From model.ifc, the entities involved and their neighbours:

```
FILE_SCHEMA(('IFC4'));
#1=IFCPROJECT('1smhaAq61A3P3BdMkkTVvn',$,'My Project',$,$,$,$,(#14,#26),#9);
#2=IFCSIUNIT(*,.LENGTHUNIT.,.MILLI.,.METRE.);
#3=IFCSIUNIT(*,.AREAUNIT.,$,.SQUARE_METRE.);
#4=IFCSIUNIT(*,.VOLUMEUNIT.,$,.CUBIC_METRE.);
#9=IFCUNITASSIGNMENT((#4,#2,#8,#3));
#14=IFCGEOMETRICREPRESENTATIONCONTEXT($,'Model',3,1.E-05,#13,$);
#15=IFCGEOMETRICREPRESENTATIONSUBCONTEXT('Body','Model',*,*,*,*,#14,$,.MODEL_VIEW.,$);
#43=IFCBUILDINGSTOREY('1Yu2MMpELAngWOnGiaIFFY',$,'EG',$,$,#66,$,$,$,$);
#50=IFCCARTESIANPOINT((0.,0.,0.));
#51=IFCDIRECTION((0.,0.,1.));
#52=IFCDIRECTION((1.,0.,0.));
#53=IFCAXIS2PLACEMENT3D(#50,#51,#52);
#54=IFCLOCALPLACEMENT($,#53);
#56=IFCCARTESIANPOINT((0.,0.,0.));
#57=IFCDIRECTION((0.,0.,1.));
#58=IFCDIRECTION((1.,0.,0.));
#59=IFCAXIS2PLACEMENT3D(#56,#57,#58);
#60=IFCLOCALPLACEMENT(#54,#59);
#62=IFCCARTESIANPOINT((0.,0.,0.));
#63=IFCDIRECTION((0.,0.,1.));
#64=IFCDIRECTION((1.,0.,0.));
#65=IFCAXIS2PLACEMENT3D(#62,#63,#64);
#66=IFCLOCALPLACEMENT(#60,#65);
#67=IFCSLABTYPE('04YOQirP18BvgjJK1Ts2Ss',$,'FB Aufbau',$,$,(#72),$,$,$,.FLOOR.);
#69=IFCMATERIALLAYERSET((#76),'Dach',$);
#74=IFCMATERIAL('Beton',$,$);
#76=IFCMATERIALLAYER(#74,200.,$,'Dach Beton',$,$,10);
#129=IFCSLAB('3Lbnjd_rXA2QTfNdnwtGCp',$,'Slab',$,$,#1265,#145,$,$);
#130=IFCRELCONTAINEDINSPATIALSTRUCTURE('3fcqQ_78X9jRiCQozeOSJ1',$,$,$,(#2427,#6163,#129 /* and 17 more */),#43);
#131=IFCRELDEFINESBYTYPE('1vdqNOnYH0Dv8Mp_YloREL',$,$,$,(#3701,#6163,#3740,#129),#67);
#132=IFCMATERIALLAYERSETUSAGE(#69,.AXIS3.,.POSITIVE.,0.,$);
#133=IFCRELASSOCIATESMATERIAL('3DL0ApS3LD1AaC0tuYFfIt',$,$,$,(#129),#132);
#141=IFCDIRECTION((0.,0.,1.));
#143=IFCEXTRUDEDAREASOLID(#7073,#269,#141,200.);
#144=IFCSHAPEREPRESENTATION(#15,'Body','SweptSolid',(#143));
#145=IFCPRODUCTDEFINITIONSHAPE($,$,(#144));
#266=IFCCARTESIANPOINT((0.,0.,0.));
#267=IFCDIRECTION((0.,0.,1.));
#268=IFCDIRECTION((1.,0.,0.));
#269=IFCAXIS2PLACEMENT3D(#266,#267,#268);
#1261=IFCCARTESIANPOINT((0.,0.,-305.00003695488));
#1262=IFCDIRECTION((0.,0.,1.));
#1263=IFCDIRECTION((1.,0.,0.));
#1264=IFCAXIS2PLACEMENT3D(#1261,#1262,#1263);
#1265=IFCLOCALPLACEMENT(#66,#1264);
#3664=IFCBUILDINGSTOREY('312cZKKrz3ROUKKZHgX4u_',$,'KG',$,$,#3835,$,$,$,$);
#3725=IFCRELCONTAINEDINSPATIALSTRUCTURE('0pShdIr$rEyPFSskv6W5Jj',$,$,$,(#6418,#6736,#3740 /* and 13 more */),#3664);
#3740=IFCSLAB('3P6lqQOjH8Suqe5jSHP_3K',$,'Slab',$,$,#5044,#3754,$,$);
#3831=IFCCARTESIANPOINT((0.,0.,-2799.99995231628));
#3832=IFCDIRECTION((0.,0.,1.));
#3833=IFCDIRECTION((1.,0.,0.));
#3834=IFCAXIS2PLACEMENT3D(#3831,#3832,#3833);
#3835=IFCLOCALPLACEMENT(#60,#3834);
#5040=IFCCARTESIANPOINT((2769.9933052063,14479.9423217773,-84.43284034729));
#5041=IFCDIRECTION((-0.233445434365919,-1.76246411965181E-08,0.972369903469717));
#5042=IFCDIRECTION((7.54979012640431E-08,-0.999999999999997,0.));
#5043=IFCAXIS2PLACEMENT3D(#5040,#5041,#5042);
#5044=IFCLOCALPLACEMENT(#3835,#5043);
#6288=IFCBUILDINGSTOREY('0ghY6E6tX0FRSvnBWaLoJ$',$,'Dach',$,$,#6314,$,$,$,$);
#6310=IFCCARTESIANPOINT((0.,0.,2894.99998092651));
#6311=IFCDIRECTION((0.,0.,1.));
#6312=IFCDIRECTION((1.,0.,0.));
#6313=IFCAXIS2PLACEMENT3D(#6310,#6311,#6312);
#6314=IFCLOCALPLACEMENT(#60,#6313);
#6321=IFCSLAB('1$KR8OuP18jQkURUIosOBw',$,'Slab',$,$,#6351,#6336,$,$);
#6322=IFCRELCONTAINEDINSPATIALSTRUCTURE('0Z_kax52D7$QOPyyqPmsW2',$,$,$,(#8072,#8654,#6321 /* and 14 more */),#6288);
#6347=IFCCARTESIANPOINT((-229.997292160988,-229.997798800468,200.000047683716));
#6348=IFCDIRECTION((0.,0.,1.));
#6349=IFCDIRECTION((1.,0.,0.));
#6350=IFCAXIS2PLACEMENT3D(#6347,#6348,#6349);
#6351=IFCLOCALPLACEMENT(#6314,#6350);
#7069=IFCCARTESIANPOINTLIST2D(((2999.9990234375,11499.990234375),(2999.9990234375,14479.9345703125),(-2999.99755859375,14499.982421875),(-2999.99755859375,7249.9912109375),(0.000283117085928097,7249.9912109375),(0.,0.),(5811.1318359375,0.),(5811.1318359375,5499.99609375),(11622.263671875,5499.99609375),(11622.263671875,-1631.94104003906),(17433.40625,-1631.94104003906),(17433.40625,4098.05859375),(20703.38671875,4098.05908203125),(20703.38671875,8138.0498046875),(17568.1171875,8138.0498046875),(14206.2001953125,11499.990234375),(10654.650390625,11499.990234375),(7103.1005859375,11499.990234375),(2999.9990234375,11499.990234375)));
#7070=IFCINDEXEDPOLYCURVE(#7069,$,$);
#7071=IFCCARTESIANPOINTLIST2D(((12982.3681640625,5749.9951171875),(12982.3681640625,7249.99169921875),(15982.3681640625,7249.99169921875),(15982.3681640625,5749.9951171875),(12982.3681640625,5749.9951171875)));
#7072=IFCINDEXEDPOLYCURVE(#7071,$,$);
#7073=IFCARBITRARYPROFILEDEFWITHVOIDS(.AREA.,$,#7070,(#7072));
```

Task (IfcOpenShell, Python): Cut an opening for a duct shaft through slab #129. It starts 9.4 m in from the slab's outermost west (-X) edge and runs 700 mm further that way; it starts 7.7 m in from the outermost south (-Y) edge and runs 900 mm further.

```python
import numpy as np
import ifcopenshell
import ifcopenshell.api.feature
import ifcopenshell.api.geometry
import ifcopenshell.api.root
import ifcopenshell.geom
import ifcopenshell.util.placement
import ifcopenshell.util.representation
import ifcopenshell.util.shape
import ifcopenshell.util.unit

model = ifcopenshell.open("model.ifc")
unit_scale = ifcopenshell.util.unit.calculate_unit_scale(model)
settings = ifcopenshell.geom.settings()


def volume(element):
    """Net volume in cubic metres, openings subtracted."""
    shape = ifcopenshell.geom.create_shape(settings, element)
    return ifcopenshell.util.shape.get_volume(shape.geometry)


slab = model.by_guid("3Lbnjd_rXA2QTfNdnwtGCp")
before = volume(slab)

# Extent in the slab's own axes, in metres. The edges named are its -X and -Y sides.
slab_shape = ifcopenshell.geom.create_shape(settings, slab)
vertices = ifcopenshell.util.shape.get_vertices(slab_shape.geometry)
x_min, y_min, bottom = vertices.min(axis=0)
top = vertices[:, 2].max()

opening = ifcopenshell.api.root.create_entity(model, ifc_class="IfcOpeningElement", name="Duct shaft opening", predefined_type="OPENING")
context = ifcopenshell.util.representation.get_context(model, "Model", "Body", "MODEL_VIEW")
width, depth = 0.7, 0.9
outline = [(0.0, 0.0), (width, 0.0), (width, depth), (0.0, depth), (0.0, 0.0)]
# Overshoot both faces by 50 mm so the cut is clean.
shape = ifcopenshell.api.geometry.add_slab_representation(
    model, context=context, depth=top - bottom + 0.1, polyline=outline
)
ifcopenshell.api.geometry.assign_representation(model, product=opening, representation=shape)

matrix = ifcopenshell.util.placement.get_local_placement(slab.ObjectPlacement)
matrix[:, 3] = matrix @ np.append(np.array([x_min + 9.4, y_min + 7.7, bottom - 0.05]) / unit_scale, 1.0)
ifcopenshell.api.geometry.edit_object_placement(model, product=opening, matrix=matrix, is_si=False)
ifcopenshell.api.feature.add_feature(model, feature=opening, element=slab)

after = volume(slab)

print(f"slab volume {before:.3f} -> {after:.3f} m3")

model.write("model_updated.ifc")
```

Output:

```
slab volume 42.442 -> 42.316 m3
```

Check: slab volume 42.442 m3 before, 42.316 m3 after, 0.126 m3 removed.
